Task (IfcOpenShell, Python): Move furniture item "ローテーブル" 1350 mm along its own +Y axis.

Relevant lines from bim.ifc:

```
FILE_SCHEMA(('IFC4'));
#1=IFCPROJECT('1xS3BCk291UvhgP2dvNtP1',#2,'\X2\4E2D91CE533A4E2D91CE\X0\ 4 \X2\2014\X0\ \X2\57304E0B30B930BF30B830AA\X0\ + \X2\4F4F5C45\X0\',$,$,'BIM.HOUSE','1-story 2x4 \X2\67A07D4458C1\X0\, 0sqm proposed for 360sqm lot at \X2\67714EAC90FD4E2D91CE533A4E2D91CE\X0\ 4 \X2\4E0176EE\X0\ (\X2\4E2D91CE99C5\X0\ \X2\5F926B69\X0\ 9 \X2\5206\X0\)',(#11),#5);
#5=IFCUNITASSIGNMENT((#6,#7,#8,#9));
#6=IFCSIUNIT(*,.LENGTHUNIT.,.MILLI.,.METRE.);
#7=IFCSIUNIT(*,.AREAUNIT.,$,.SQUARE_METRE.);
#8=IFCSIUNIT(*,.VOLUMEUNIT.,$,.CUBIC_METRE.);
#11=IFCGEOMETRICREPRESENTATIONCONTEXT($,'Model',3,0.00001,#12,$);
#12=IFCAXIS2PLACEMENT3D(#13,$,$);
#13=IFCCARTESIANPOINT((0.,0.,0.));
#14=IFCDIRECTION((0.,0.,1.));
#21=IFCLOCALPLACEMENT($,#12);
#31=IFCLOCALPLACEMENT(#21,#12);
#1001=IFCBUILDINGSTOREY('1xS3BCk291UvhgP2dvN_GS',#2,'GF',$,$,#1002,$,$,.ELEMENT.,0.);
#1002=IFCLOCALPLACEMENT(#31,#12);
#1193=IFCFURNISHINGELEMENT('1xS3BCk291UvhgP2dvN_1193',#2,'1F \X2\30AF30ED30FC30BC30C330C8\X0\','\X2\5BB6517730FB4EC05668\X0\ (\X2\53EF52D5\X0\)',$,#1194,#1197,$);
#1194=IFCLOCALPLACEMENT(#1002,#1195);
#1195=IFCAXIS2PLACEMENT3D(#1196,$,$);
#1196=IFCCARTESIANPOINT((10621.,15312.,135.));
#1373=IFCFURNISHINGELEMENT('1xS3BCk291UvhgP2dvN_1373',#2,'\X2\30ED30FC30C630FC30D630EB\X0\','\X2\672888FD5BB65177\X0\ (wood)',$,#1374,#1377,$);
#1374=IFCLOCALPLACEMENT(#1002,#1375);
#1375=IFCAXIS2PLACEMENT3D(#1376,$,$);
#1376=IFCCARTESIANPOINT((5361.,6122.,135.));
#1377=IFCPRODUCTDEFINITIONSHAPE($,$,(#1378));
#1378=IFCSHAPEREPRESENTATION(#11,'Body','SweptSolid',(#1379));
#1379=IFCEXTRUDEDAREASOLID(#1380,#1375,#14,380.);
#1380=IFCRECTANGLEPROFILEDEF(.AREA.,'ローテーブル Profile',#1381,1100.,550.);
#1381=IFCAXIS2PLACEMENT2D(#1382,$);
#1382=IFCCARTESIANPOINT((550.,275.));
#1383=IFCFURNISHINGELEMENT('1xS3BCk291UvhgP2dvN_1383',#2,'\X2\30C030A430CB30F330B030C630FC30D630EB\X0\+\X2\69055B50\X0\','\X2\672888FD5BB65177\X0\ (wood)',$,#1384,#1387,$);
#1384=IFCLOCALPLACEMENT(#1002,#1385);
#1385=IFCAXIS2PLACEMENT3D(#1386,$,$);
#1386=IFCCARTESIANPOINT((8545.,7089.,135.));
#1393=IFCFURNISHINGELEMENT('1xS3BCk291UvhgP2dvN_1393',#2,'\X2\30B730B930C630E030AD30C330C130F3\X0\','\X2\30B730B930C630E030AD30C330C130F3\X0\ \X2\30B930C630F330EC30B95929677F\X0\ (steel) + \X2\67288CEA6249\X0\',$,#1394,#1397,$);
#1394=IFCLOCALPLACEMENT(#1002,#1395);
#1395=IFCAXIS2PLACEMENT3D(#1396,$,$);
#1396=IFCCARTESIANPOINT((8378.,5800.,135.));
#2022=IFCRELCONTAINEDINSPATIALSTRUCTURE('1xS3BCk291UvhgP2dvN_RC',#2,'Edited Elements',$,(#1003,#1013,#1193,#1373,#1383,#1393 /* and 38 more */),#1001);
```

```python
import ifcopenshell
import ifcopenshell.api.geometry
import ifcopenshell.util.placement
import ifcopenshell.util.unit

model = ifcopenshell.open("bim.ifc")
unit_scale = ifcopenshell.util.unit.calculate_unit_scale(model)

item = model.by_guid("1xS3BCk291UvhgP2dvN_1373")
matrix = ifcopenshell.util.placement.get_local_placement(item.ObjectPlacement)
matrix[:3, 3] += matrix[:3, 1] * 1.35 / unit_scale
ifcopenshell.api.geometry.edit_object_placement(model, product=item, matrix=matrix, is_si=False)

print(ifcopenshell.util.placement.get_local_placement(item.ObjectPlacement).round(3) + 0.0)

model.write("bim_v2.ifc")
```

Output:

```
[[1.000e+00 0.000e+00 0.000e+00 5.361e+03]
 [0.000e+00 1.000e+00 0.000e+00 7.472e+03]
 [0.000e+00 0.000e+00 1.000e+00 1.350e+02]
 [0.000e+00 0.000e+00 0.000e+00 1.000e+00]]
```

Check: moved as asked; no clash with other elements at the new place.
